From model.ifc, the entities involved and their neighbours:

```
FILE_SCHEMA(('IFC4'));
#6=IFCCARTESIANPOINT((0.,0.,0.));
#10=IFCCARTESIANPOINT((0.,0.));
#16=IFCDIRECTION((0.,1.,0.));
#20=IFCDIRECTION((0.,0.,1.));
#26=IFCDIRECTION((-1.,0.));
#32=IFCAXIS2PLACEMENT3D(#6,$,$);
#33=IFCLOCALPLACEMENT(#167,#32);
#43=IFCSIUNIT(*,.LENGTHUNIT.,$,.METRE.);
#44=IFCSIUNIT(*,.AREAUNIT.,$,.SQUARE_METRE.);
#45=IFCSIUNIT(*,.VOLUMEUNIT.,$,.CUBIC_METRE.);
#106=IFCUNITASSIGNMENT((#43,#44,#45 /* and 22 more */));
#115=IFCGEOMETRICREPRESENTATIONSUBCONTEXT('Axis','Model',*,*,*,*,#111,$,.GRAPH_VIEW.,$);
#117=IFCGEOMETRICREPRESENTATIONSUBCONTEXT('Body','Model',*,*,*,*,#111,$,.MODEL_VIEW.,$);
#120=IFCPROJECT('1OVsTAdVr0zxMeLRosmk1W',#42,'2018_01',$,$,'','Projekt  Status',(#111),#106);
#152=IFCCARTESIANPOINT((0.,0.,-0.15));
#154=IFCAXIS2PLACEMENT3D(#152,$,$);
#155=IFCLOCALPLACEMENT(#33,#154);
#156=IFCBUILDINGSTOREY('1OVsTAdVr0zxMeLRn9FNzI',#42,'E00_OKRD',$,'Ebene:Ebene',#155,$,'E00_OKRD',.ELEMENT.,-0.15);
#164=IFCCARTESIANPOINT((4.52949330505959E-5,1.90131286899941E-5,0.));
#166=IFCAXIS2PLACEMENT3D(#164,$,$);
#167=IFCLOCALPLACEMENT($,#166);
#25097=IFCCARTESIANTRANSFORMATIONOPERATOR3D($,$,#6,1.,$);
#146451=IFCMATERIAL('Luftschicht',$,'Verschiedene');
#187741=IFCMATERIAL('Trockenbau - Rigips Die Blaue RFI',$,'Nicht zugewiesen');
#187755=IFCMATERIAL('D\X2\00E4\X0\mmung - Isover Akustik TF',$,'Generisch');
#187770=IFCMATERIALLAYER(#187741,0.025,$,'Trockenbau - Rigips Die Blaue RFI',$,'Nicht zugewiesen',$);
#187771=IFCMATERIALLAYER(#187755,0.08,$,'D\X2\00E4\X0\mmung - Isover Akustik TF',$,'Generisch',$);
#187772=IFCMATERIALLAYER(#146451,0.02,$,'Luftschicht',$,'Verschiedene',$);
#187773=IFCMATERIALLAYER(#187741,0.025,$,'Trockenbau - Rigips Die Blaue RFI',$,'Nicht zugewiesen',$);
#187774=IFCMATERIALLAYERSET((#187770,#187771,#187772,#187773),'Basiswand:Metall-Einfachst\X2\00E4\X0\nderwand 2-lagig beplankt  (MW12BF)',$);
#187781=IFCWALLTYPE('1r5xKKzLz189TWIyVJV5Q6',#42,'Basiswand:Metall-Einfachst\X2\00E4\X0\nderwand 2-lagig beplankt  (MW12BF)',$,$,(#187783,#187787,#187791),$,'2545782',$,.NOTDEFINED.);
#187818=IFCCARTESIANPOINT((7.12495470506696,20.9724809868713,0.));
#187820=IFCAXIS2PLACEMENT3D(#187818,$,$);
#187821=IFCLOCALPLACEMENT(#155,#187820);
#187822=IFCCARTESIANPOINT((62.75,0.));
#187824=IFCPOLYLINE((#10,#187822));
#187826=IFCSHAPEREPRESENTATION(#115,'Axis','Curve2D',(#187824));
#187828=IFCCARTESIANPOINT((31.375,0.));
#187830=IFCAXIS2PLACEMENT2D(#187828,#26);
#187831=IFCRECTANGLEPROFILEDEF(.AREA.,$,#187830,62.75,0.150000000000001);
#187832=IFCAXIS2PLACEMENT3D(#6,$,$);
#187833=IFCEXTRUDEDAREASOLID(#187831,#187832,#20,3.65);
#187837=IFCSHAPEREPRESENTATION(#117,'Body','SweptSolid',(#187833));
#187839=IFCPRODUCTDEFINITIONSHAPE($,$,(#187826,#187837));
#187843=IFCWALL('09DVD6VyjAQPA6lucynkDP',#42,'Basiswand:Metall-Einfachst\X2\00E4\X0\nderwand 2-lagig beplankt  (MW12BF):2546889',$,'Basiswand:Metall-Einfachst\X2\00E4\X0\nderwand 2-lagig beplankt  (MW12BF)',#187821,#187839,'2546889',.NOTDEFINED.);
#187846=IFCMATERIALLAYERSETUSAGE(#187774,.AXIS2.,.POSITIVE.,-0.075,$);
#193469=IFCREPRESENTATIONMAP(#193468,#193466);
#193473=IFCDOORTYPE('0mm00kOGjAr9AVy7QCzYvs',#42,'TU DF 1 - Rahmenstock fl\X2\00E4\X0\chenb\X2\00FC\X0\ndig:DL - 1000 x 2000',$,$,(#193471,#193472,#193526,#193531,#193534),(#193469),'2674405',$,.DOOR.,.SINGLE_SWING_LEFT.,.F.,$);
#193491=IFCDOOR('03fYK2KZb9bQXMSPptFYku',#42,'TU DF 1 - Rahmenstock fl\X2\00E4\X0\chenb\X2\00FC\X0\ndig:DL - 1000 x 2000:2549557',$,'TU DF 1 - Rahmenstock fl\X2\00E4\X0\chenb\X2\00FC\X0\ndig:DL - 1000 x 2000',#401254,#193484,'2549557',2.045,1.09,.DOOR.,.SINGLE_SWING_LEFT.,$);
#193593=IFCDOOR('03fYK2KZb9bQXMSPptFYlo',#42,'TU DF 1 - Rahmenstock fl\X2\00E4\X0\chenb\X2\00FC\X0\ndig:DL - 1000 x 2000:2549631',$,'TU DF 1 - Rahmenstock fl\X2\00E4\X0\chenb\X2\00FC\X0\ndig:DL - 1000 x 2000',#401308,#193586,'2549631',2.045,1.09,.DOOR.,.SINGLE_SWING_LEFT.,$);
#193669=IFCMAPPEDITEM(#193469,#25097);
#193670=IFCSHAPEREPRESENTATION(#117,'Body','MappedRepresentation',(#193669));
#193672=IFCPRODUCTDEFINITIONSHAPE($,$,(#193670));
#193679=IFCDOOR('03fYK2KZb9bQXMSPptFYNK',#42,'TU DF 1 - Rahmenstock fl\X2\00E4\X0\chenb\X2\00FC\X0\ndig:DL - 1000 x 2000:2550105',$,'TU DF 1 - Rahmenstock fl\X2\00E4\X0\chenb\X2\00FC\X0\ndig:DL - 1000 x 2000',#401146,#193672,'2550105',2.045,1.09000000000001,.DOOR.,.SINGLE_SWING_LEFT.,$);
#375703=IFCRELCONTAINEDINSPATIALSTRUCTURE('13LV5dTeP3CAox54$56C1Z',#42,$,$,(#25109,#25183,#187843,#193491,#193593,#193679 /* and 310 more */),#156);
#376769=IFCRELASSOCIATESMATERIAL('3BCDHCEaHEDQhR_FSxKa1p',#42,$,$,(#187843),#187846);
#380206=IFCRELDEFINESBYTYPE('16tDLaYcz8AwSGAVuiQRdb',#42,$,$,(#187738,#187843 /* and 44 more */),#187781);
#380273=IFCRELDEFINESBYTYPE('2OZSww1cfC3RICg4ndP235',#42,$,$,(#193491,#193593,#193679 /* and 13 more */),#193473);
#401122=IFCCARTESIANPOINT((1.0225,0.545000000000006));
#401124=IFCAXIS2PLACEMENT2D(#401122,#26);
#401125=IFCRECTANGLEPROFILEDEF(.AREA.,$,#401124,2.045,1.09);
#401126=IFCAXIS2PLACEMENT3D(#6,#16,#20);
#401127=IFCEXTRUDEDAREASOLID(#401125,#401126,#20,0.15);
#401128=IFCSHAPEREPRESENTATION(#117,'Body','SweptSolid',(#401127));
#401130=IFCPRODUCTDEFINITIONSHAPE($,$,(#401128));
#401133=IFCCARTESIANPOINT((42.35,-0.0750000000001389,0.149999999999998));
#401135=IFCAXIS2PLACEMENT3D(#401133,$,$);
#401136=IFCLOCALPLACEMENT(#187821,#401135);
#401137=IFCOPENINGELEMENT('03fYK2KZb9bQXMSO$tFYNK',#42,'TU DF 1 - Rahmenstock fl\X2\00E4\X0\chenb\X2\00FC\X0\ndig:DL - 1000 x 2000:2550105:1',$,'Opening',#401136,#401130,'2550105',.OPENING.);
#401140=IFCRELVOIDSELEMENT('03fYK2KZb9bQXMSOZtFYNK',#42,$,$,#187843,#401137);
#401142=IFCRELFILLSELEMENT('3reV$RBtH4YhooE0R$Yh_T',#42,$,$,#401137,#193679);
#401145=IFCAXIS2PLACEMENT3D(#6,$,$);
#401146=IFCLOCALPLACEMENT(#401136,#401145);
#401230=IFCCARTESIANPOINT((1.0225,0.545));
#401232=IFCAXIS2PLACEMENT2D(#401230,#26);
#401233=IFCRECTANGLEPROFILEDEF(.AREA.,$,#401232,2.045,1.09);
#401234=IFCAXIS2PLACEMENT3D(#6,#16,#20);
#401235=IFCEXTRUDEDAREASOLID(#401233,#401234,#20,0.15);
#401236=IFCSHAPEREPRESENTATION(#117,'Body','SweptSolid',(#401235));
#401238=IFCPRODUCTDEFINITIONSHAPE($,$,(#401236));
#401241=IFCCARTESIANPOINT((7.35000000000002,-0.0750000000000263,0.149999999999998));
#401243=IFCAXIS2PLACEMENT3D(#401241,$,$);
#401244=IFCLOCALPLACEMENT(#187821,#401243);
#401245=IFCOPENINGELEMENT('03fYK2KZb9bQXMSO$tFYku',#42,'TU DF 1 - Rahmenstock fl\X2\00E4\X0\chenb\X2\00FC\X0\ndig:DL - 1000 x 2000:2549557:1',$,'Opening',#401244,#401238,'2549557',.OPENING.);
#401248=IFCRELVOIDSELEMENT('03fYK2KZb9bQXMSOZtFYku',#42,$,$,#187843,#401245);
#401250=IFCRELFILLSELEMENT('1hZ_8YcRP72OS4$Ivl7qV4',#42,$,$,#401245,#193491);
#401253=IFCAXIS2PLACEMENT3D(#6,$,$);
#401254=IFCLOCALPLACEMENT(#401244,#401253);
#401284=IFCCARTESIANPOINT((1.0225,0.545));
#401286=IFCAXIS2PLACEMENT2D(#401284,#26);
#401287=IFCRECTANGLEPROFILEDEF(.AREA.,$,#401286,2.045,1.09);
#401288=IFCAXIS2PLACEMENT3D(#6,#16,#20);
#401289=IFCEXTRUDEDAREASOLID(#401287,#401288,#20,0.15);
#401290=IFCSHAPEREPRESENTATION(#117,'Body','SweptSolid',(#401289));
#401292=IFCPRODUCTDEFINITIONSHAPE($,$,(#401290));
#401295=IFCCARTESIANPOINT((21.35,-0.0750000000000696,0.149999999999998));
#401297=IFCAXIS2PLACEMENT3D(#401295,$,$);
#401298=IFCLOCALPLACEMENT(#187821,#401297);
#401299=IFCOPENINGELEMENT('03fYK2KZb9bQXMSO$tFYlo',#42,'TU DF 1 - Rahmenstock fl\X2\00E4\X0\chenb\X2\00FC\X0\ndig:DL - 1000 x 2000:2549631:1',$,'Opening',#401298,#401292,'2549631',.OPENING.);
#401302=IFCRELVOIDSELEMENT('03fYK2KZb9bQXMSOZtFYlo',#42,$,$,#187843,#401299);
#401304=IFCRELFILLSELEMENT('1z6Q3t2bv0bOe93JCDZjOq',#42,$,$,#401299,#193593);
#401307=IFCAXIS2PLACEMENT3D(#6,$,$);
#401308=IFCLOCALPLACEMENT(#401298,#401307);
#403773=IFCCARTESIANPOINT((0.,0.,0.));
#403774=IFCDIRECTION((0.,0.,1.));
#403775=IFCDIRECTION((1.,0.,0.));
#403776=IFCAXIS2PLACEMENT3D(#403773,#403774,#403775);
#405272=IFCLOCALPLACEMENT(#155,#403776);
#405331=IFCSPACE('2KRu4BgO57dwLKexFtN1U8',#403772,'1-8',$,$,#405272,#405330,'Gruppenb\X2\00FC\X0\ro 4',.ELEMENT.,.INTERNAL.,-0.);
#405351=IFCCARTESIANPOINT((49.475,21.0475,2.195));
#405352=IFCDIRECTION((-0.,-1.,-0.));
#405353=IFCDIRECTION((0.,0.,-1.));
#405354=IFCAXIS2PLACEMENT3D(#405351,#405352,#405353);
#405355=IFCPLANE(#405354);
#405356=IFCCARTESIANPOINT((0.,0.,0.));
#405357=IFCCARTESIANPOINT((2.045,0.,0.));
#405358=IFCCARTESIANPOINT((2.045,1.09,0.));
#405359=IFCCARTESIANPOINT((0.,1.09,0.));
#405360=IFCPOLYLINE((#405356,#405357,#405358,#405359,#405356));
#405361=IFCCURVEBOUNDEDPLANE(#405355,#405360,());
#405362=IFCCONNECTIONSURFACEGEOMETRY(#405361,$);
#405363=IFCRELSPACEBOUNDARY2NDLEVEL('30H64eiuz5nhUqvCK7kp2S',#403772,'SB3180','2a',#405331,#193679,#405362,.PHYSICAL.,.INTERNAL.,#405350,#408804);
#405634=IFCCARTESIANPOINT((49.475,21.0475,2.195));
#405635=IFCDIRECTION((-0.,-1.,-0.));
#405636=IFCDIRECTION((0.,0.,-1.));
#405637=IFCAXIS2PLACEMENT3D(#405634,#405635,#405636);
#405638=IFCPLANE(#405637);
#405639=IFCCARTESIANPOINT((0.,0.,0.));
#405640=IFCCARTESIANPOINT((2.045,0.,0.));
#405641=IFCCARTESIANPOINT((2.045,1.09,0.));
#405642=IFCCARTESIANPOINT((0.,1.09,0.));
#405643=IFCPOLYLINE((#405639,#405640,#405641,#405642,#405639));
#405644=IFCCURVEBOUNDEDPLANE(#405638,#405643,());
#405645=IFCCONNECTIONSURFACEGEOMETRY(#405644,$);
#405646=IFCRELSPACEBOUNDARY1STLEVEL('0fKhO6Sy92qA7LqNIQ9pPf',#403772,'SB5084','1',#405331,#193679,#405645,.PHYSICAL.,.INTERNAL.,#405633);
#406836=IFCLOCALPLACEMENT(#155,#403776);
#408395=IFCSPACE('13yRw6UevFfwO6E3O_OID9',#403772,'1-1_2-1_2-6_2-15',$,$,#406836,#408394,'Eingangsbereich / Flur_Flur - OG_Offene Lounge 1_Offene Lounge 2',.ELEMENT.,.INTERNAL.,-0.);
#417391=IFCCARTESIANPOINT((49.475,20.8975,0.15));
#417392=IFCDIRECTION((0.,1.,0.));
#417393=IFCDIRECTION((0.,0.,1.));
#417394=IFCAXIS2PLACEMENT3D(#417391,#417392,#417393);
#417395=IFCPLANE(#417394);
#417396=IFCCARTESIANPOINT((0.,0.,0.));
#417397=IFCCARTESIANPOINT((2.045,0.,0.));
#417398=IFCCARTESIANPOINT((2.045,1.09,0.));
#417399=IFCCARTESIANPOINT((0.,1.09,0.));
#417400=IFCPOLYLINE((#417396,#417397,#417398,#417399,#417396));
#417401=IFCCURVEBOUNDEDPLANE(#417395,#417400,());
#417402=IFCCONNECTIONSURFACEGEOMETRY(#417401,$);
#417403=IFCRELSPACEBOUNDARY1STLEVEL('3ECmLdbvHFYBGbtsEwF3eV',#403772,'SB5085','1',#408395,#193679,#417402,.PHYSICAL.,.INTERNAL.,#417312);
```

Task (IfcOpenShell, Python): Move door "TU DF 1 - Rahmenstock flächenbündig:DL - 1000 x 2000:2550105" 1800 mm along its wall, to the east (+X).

```python
import numpy as np
import ifcopenshell
import ifcopenshell.api.geometry
import ifcopenshell.util.placement
import ifcopenshell.util.unit

model = ifcopenshell.open("model.ifc")
unit_scale = ifcopenshell.util.unit.calculate_unit_scale(model)

door = model.by_guid("03fYK2KZb9bQXMSPptFYNK")
opening = door.FillsVoids[0].RelatingOpeningElement
wall = opening.VoidsElements[0].RelatingBuildingElement

wall_matrix = ifcopenshell.util.placement.get_local_placement(wall.ObjectPlacement)
shift = wall_matrix[:3, 0] * 1.8 / unit_scale
before = ifcopenshell.util.placement.get_local_placement(door.ObjectPlacement)[:3, 3].copy()

# The door is placed relative to its opening, so it follows when the opening moves.
matrix = ifcopenshell.util.placement.get_local_placement(opening.ObjectPlacement)
matrix[:3, 3] += shift
ifcopenshell.api.geometry.edit_object_placement(
    model, product=opening, matrix=matrix, is_si=False, should_transform_children=True
)

# Space boundary surfaces are stored in each space's coordinates; move them too.
for rel in door.ProvidesBoundaries:
    if not rel.ConnectionGeometry:
        continue
    surface = rel.ConnectionGeometry.SurfaceOnRelatingElement.BasisSurface
    space_matrix = ifcopenshell.util.placement.get_local_placement(rel.RelatingSpace.ObjectPlacement)
    point = np.array(surface.Position.Location.Coordinates) + space_matrix[:3, :3].T @ shift
    surface.Position = model.createIfcAxis2Placement3D(
        model.createIfcCartesianPoint(point.tolist()), surface.Position.Axis, surface.Position.RefDirection
    )

after = ifcopenshell.util.placement.get_local_placement(door.ObjectPlacement)[:3, 3]
print("door moved by", (after - before).round(3) + 0.0)

model.write("model-out.ifc")
```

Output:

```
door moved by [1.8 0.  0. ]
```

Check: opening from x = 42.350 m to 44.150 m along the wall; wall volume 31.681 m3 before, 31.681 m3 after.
